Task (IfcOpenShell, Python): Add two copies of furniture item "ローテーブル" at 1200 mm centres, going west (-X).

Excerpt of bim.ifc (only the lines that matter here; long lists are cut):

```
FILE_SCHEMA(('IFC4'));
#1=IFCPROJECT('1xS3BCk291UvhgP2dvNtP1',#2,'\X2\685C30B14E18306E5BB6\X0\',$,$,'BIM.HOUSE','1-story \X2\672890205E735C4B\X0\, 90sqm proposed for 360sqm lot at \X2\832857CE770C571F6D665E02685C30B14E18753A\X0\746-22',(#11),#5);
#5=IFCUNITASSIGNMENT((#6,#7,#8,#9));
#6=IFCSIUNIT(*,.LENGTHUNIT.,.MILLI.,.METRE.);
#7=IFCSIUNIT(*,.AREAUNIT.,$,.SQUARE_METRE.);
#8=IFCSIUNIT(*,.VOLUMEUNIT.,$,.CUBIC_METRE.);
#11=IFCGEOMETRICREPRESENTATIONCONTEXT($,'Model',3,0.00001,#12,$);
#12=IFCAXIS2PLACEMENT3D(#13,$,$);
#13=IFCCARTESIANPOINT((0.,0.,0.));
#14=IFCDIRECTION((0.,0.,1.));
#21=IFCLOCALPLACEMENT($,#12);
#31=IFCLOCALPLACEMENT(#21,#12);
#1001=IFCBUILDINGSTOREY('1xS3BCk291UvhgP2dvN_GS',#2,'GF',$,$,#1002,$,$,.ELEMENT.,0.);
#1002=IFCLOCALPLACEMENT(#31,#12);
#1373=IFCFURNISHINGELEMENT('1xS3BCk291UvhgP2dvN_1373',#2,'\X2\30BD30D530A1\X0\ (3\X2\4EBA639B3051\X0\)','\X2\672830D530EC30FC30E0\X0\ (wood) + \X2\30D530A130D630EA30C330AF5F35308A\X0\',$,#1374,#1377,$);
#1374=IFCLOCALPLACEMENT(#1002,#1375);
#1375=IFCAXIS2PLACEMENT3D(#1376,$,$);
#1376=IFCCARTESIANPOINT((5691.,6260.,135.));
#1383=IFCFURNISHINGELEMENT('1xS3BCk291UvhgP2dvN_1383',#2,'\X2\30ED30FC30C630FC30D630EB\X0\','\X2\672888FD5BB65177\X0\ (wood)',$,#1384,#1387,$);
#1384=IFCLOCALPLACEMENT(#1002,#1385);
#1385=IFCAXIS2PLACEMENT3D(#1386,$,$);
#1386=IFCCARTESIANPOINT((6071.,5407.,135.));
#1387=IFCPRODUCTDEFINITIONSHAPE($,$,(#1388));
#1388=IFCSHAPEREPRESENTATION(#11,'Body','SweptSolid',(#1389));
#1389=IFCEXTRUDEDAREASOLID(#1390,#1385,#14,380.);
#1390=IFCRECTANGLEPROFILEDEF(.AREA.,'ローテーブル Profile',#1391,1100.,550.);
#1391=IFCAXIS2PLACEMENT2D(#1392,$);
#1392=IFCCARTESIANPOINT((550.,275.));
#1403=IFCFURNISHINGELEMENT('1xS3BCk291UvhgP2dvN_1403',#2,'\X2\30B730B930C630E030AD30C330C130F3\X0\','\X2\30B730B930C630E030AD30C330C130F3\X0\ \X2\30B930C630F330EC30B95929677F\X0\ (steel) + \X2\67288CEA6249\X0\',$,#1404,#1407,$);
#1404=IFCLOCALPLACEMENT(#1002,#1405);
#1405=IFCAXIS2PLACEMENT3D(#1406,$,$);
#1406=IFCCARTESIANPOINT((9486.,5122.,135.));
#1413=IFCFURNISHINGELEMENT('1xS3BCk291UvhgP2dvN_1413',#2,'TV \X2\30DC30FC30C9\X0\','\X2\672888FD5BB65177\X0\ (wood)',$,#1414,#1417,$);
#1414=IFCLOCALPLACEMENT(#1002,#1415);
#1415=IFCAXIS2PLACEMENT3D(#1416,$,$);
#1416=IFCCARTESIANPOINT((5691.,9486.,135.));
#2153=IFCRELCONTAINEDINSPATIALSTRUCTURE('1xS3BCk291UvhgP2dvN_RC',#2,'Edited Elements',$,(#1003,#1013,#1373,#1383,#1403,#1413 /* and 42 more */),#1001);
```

```python
import numpy as np
import ifcopenshell
import ifcopenshell.api.geometry
import ifcopenshell.api.root
import ifcopenshell.util.element
import ifcopenshell.util.placement

model = ifcopenshell.open("bim.ifc")


def reuse_history(source, copy):
    """copy_class also copies each property set's owner history, people and application; keep the originals."""
    for rel in copy.IsDefinedBy:
        if rel.is_a("IfcRelDefinesByProperties") and (history := rel.RelatingPropertyDefinition.OwnerHistory):
            rel.RelatingPropertyDefinition.OwnerHistory = source.OwnerHistory
            ifcopenshell.util.element.remove_deep2(model, history)


source = model.by_guid("1xS3BCk291UvhgP2dvN_1383")
base = ifcopenshell.util.placement.get_local_placement(source.ObjectPlacement)
step = np.array([-1.0, 0.0, 0.0]) * 1200.0

for i in range(1, 3):
    copy = ifcopenshell.api.root.copy_class(model, product=source)
    copy.Representation = ifcopenshell.util.element.copy_deep(
        model, source.Representation, exclude=["IfcGeometricRepresentationContext", "IfcRepresentationMap"]
    )
    reuse_history(source, copy)
    matrix = base.copy()
    matrix[:3, 3] += i * step
    print("added at", matrix[:3, 3].round(3) + 0.0)
    ifcopenshell.api.geometry.edit_object_placement(model, product=copy, matrix=matrix, is_si=False)

model.write("bim_rev.ifc")
```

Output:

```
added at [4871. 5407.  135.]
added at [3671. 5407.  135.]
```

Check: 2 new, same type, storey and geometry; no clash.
